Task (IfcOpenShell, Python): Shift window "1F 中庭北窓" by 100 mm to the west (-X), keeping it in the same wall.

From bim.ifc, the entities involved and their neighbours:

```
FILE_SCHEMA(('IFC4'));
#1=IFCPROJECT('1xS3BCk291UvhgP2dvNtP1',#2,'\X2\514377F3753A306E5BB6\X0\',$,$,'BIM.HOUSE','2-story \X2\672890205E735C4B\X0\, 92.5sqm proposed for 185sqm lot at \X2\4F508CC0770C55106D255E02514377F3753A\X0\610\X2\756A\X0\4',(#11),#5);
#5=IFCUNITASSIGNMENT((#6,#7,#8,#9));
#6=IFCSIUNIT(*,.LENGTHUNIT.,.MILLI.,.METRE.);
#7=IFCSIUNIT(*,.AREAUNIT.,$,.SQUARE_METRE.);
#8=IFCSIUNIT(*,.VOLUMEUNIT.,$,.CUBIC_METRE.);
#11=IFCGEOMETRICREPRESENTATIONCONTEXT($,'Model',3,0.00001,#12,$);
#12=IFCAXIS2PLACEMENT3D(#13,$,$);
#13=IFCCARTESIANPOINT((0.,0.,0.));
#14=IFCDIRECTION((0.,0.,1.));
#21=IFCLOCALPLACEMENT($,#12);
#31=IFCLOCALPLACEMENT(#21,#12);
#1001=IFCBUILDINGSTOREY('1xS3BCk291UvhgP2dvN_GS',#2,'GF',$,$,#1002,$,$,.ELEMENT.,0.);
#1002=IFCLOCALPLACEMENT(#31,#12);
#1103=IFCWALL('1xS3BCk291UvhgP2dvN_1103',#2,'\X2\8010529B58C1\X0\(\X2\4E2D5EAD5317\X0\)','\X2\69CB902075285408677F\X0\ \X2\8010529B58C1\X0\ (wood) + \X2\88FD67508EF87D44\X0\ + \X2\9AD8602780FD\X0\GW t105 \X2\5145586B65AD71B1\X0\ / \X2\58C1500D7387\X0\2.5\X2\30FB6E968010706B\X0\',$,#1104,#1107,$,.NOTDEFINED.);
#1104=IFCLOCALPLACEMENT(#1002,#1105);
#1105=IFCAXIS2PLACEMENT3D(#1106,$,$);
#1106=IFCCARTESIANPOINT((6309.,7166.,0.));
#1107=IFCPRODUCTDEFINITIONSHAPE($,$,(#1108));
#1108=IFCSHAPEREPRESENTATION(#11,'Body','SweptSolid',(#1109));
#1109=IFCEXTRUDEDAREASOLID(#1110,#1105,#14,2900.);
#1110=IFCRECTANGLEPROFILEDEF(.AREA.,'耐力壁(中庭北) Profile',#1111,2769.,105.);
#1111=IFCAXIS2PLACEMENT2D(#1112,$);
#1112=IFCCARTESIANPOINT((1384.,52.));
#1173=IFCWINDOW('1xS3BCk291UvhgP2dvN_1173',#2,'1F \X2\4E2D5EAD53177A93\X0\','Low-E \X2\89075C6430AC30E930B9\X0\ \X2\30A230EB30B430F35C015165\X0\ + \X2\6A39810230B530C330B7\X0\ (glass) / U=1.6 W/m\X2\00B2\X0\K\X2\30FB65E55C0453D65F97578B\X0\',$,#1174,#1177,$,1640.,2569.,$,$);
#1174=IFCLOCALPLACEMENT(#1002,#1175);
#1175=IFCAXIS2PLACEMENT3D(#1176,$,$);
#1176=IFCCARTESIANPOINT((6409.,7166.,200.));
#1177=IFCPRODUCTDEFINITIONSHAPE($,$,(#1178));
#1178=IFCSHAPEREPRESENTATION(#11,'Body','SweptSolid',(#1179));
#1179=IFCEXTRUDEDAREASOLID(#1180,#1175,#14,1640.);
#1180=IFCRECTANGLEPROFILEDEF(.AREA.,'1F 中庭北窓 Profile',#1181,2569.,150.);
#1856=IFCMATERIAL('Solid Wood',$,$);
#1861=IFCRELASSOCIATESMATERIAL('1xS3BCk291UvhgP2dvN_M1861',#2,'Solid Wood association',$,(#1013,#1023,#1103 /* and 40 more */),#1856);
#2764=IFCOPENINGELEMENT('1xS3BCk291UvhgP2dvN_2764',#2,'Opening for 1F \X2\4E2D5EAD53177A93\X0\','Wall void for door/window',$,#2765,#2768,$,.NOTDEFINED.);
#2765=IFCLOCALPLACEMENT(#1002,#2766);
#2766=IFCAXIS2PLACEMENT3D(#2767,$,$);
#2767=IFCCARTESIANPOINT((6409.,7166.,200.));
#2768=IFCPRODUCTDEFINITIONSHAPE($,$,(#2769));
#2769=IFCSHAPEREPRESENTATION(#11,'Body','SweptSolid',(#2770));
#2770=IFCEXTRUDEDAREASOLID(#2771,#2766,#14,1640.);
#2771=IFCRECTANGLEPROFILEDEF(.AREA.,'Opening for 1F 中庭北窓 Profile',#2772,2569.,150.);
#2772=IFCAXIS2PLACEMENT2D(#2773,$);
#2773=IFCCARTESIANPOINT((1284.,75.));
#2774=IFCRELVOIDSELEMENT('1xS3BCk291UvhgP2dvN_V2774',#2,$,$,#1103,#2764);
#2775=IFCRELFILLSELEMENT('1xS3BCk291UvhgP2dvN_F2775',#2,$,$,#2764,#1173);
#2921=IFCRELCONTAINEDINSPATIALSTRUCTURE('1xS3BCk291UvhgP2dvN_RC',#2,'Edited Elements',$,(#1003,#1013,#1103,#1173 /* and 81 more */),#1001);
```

```python
import ifcopenshell
import ifcopenshell.api.geometry
import ifcopenshell.util.placement
import ifcopenshell.util.unit

model = ifcopenshell.open("bim.ifc")
unit_scale = ifcopenshell.util.unit.calculate_unit_scale(model)

window = model.by_id(1173)
opening = window.FillsVoids[0].RelatingOpeningElement
wall = opening.VoidsElements[0].RelatingBuildingElement

wall_matrix = ifcopenshell.util.placement.get_local_placement(wall.ObjectPlacement)
shift = wall_matrix[:3, 0] * -0.1 / unit_scale
before = ifcopenshell.util.placement.get_local_placement(window.ObjectPlacement)[:3, 3].copy()

# The window is not placed relative to its opening, so move both.
for product in (opening, window):
    matrix = ifcopenshell.util.placement.get_local_placement(product.ObjectPlacement)
    matrix[:3, 3] += shift
    ifcopenshell.api.geometry.edit_object_placement(model, product=product, matrix=matrix, is_si=False)

after = ifcopenshell.util.placement.get_local_placement(window.ObjectPlacement)[:3, 3]
print("window moved by", (after - before).round(3) + 0.0)

model.write("bim_rev.ifc")
```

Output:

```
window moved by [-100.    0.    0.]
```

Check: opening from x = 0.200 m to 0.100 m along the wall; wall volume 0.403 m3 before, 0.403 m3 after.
